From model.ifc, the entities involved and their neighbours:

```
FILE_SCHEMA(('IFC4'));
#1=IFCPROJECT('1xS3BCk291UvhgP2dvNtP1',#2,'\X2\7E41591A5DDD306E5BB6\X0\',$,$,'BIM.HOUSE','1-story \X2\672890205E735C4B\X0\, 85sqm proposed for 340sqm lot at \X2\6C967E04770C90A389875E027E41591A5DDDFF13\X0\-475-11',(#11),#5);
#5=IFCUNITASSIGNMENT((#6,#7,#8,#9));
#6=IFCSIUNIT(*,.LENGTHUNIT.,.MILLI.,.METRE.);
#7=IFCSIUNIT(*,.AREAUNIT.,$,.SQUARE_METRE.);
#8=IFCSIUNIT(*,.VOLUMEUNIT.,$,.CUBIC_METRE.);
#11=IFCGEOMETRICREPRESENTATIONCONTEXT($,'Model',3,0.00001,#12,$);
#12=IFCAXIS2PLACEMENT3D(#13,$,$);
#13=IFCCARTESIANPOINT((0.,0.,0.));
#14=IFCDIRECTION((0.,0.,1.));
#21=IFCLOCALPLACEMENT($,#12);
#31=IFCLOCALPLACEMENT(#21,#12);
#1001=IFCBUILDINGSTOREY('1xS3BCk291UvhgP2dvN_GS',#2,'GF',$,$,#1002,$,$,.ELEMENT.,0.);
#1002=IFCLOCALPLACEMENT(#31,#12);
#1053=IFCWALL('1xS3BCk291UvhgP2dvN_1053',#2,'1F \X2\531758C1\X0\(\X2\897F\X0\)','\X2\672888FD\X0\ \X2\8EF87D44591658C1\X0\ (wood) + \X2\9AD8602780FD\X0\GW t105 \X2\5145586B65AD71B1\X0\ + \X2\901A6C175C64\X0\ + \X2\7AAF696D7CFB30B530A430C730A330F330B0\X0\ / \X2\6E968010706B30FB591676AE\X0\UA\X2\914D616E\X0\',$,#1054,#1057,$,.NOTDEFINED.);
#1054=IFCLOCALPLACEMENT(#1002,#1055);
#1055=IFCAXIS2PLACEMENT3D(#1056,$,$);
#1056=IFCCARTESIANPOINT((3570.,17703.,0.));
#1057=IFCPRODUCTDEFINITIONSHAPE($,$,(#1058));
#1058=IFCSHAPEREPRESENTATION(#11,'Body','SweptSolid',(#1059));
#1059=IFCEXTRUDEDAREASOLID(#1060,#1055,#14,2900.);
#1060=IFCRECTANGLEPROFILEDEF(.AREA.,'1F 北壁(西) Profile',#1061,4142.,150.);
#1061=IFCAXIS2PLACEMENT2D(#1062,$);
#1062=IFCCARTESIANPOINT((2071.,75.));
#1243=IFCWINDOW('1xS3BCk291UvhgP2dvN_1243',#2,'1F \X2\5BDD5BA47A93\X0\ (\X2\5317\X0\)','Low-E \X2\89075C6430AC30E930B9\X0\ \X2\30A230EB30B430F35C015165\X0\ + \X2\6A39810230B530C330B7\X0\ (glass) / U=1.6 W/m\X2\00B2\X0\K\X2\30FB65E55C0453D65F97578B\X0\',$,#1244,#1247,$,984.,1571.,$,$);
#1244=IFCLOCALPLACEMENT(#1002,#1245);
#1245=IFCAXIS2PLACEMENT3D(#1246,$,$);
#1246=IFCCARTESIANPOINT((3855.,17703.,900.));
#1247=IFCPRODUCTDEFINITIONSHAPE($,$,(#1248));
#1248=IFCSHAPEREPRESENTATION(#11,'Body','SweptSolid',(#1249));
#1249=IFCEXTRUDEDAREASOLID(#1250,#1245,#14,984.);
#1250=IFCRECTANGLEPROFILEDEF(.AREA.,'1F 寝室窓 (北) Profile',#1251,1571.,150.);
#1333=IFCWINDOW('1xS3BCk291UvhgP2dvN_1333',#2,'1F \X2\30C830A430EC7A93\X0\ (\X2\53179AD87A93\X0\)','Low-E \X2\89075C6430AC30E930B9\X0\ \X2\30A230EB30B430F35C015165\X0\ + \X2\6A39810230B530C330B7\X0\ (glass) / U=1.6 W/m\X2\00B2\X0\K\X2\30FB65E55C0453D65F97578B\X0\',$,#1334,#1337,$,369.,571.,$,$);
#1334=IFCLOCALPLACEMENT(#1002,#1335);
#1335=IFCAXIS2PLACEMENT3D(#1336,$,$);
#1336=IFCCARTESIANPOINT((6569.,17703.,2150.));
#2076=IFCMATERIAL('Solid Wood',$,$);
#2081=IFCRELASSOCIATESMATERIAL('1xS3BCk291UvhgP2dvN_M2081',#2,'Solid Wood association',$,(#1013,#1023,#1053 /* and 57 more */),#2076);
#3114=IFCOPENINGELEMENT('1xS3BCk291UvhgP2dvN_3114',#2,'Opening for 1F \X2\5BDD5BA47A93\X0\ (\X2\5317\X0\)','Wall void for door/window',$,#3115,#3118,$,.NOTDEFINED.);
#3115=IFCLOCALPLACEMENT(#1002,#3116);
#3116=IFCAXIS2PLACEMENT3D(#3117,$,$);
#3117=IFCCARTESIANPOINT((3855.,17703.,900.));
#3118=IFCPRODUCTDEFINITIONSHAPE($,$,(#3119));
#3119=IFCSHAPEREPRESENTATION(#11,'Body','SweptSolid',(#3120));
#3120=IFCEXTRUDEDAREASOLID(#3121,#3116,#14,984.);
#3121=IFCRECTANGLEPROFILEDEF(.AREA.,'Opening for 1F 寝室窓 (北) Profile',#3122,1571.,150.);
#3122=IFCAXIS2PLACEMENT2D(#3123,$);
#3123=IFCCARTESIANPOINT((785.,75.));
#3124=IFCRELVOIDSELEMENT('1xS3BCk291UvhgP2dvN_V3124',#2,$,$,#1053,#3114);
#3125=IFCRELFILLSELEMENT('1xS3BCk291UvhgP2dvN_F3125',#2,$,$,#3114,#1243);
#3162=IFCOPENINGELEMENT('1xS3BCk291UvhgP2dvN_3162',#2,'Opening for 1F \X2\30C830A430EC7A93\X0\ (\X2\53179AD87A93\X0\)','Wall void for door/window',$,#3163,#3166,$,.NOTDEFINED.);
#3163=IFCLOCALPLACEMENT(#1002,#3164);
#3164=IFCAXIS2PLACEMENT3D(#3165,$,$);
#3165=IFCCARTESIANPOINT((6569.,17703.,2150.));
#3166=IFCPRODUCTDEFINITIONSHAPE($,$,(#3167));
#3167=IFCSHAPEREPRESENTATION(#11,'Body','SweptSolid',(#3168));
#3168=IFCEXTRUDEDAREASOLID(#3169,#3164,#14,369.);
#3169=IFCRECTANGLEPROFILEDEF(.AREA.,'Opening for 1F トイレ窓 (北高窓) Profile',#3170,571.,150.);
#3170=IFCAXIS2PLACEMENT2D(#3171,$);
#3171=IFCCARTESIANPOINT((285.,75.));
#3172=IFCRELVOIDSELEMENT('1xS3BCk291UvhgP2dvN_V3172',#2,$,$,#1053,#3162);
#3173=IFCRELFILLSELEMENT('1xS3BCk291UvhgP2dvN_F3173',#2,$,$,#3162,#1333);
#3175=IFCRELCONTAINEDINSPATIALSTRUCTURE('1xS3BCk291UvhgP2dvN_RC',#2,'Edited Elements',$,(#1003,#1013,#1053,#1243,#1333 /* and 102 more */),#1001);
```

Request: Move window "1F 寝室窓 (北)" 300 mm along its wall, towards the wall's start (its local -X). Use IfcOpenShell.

```python
import ifcopenshell
import ifcopenshell.api.geometry
import ifcopenshell.util.placement
import ifcopenshell.util.unit

model = ifcopenshell.open("model.ifc")
unit_scale = ifcopenshell.util.unit.calculate_unit_scale(model)

window = model.by_guid("1xS3BCk291UvhgP2dvN_1243")
opening = window.FillsVoids[0].RelatingOpeningElement
wall = opening.VoidsElements[0].RelatingBuildingElement

wall_matrix = ifcopenshell.util.placement.get_local_placement(wall.ObjectPlacement)
shift = wall_matrix[:3, 0] * -0.3 / unit_scale
before = ifcopenshell.util.placement.get_local_placement(window.ObjectPlacement)[:3, 3].copy()

# The window is not placed relative to its opening, so move both.
for product in (opening, window):
    matrix = ifcopenshell.util.placement.get_local_placement(product.ObjectPlacement)
    matrix[:3, 3] += shift
    ifcopenshell.api.geometry.edit_object_placement(model, product=product, matrix=matrix, is_si=False)

after = ifcopenshell.util.placement.get_local_placement(window.ObjectPlacement)[:3, 3]
print("window moved by", (after - before).round(3) + 0.0)

model.write("model_rev.ifc")
```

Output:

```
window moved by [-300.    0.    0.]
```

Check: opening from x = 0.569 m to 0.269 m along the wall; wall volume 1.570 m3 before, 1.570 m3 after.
